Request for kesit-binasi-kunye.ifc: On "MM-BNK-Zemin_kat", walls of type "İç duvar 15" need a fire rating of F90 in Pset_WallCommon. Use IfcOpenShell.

First a look at what the model holds.

```python
import ifcopenshell
import ifcopenshell.util.element

model = ifcopenshell.open("kesit-binasi-kunye.ifc")
print(model.schema)
storey = next(s for s in model.by_type("IfcBuildingStorey") if s.Name == "MM-BNK-Zemin_kat")
walls = [e for e in ifcopenshell.util.element.get_decomposition(storey) if e.is_a("IfcWall")]
seen = {}
for e in walls:
    element_type = ifcopenshell.util.element.get_type(e)
    key = (element_type.Name if element_type != e and element_type else None, ifcopenshell.util.element.get_pset(e, "Pset_WallCommon", "FireRating"))
    seen[key] = seen.get(key, 0) + 1
for (name, value), count in sorted(seen.items(), key=str):
    print(count, "x", name, "|", value)
```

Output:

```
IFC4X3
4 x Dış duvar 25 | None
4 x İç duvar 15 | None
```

```python
import ifcopenshell
import ifcopenshell.api.pset
import ifcopenshell.util.element

model = ifcopenshell.open("kesit-binasi-kunye.ifc")

storey = next(s for s in model.by_type("IfcBuildingStorey") if s.Name == "MM-BNK-Zemin_kat")
walls = [e for e in ifcopenshell.util.element.get_decomposition(storey) if e.is_a("IfcWall")]

count = 0
for e in walls:
    element_type = ifcopenshell.util.element.get_type(e)
    if element_type in (None, e) or element_type.Name != "İç duvar 15":
        continue
    # add_pset returns the element's existing set when there is one.
    pset = ifcopenshell.api.pset.add_pset(model, product=e, name="Pset_WallCommon")
    ifcopenshell.api.pset.edit_pset(model, pset=pset, properties={"FireRating": "F90"})
    count += 1

print(count, "walls updated")

model.write("kesit-binasi-kunye_updated.ifc")
```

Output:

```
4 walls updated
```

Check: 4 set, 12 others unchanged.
